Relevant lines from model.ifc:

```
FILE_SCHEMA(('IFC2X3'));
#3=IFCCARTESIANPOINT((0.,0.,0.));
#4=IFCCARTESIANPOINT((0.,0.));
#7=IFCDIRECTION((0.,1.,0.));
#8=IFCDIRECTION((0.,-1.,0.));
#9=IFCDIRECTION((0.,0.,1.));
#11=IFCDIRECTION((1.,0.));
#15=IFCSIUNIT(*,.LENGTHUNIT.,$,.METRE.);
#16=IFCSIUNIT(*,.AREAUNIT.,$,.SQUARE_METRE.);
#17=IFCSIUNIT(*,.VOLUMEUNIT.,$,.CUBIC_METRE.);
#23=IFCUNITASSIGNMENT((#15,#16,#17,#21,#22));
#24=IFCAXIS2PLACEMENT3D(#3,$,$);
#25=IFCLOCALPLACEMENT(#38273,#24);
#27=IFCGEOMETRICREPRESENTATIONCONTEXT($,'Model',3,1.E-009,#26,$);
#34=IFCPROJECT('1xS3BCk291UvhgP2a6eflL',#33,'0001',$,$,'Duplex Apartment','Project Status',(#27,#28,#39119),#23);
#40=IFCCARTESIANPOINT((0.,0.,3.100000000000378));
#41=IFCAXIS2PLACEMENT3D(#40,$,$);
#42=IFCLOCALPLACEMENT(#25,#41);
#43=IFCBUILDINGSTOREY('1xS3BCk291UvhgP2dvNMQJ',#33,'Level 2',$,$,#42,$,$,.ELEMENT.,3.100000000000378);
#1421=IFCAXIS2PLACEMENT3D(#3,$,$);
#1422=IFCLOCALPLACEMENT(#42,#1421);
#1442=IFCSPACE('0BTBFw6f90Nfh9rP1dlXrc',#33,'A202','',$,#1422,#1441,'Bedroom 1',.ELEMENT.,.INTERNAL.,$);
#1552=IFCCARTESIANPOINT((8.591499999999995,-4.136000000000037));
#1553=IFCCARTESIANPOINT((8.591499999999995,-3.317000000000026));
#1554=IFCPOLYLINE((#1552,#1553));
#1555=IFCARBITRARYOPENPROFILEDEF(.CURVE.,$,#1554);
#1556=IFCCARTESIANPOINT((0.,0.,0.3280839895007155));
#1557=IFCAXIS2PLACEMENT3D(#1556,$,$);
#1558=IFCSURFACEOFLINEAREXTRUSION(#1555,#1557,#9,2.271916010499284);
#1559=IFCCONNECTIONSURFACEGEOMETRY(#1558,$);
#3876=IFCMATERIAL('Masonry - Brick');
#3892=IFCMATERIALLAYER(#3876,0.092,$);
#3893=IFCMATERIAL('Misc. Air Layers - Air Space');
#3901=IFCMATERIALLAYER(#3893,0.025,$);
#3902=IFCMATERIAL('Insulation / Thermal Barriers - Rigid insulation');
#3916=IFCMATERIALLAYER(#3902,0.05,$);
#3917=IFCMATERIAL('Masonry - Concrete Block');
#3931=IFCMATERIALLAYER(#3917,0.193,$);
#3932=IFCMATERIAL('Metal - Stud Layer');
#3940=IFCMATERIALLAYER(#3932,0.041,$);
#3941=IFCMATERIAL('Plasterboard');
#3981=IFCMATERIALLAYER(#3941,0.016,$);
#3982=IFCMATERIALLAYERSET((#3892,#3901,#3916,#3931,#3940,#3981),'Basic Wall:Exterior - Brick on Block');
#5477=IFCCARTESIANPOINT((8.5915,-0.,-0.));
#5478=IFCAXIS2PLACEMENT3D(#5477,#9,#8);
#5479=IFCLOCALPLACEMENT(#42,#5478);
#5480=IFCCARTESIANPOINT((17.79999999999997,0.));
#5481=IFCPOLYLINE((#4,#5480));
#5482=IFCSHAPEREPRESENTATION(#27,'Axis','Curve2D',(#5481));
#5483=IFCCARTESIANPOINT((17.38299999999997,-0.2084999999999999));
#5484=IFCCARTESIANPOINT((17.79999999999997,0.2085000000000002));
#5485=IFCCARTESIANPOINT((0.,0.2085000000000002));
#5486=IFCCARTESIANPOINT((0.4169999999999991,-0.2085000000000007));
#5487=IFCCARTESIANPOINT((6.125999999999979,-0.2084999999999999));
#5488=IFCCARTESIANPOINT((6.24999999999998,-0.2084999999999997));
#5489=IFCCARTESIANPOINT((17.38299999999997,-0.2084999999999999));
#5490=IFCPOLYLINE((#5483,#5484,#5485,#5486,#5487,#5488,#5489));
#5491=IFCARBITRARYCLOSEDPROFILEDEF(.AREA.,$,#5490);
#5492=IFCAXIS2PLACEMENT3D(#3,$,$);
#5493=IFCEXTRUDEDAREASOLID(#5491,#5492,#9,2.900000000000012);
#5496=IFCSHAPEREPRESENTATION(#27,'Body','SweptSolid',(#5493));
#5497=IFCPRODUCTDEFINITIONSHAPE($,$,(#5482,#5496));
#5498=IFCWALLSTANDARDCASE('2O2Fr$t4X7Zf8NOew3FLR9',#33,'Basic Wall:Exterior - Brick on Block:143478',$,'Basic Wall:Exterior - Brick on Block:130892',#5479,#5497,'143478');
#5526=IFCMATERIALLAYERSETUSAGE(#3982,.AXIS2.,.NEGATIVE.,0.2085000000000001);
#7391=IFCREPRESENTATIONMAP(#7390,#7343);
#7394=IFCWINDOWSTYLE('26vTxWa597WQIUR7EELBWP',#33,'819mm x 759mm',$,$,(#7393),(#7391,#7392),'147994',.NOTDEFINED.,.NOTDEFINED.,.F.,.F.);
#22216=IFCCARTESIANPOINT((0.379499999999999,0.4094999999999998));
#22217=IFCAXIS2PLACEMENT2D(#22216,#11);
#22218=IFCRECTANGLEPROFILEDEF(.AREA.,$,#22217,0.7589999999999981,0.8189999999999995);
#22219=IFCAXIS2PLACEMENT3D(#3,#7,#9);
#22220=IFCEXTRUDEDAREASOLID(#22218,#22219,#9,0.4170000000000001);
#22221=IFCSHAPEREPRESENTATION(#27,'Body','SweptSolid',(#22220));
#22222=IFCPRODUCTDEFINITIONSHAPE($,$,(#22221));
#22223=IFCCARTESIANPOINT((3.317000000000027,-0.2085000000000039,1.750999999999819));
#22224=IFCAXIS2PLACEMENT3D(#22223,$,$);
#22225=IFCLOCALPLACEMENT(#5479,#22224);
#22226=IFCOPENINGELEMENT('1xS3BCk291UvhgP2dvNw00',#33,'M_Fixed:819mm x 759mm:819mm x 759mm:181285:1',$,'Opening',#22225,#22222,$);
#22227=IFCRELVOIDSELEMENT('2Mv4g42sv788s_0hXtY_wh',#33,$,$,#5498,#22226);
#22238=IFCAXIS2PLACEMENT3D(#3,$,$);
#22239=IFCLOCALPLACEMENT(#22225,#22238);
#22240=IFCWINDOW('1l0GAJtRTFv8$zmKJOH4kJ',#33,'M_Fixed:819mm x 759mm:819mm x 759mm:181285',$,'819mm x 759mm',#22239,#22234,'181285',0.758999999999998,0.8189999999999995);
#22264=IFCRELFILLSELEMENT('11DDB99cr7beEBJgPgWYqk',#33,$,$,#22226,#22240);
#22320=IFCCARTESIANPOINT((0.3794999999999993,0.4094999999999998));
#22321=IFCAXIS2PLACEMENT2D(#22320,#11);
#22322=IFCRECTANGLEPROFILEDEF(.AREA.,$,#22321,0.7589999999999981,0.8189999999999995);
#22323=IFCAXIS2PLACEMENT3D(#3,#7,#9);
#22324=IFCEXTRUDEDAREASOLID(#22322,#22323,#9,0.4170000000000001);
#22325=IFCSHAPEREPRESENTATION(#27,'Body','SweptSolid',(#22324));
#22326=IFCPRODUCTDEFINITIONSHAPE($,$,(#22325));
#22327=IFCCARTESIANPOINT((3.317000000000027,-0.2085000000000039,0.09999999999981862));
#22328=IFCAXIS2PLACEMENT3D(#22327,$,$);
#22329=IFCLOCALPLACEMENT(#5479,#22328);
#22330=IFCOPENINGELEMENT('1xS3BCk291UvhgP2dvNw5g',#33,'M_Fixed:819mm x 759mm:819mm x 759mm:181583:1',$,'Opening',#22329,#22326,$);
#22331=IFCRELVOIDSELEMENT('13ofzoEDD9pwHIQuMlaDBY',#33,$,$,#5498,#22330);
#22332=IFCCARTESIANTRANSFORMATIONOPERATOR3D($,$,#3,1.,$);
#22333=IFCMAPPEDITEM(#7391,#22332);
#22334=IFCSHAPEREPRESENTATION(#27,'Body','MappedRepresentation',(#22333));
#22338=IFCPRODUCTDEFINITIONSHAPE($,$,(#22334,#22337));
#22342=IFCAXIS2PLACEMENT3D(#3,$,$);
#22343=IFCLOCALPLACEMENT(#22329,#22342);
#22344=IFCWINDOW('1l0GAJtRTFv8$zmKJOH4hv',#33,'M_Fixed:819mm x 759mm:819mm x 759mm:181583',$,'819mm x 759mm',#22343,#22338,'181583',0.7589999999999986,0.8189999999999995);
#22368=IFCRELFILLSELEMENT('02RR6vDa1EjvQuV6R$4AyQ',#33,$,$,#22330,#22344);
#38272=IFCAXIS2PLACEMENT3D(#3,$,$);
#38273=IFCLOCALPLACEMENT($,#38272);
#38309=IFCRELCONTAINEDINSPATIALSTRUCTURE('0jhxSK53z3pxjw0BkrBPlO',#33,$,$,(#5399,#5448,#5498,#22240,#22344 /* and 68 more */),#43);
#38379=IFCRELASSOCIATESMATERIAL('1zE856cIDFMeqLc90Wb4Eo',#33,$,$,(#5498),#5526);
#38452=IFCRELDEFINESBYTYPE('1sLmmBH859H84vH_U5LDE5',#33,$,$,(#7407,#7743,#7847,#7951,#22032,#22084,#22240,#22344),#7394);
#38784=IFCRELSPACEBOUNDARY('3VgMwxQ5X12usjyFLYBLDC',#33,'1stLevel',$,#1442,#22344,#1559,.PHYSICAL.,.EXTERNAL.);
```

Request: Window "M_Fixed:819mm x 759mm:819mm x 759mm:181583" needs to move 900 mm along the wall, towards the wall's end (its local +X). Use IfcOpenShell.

```python
import numpy as np
import ifcopenshell
import ifcopenshell.api.geometry
import ifcopenshell.util.placement
import ifcopenshell.util.unit

model = ifcopenshell.open("model.ifc")
unit_scale = ifcopenshell.util.unit.calculate_unit_scale(model)

window = model.by_guid("1l0GAJtRTFv8$zmKJOH4hv")
opening = window.FillsVoids[0].RelatingOpeningElement
wall = opening.VoidsElements[0].RelatingBuildingElement

wall_matrix = ifcopenshell.util.placement.get_local_placement(wall.ObjectPlacement)
shift = wall_matrix[:3, 0] * 0.9 / unit_scale
before = ifcopenshell.util.placement.get_local_placement(window.ObjectPlacement)[:3, 3].copy()

# The window is placed relative to its opening, so it follows when the opening moves.
matrix = ifcopenshell.util.placement.get_local_placement(opening.ObjectPlacement)
matrix[:3, 3] += shift
ifcopenshell.api.geometry.edit_object_placement(
    model, product=opening, matrix=matrix, is_si=False, should_transform_children=True
)

# Space boundary surfaces are stored in each space's coordinates; move them too.
for rel in window.ProvidesBoundaries:
    if not rel.ConnectionGeometry:
        continue
    surface = rel.ConnectionGeometry.SurfaceOnRelatingElement
    space_matrix = ifcopenshell.util.placement.get_local_placement(rel.RelatingSpace.ObjectPlacement)
    point = np.array(surface.Position.Location.Coordinates) + space_matrix[:3, :3].T @ shift
    surface.Position = model.createIfcAxis2Placement3D(
        model.createIfcCartesianPoint(point.tolist()), surface.Position.Axis, surface.Position.RefDirection
    )

after = ifcopenshell.util.placement.get_local_placement(window.ObjectPlacement)[:3, 3]
print("window moved by", (after - before).round(3) + 0.0)

model.write("model_v2.ifc")
```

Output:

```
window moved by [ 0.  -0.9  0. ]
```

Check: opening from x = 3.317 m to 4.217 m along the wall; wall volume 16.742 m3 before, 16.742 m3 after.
